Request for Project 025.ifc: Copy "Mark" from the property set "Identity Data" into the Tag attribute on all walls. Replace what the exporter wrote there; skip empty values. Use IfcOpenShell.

First a look at what the model holds.

```python
import ifcopenshell
import ifcopenshell.util.element

model = ifcopenshell.open("Project 025.ifc")
print(model.schema)
walls = model.by_type("IfcWall")
print(len(walls), "walls")
for e in walls[:8]:
    source = ifcopenshell.util.element.get_pset(e, "Identity Data", "Mark")
    target = e.Tag
    print(e.id(), repr(source), repr(target), sep=" | ")
```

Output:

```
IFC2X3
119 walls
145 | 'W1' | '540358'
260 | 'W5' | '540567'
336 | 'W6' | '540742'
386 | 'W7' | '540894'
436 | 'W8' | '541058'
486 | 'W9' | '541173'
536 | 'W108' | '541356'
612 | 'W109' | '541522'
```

```python
import ifcopenshell
import ifcopenshell.util.element

model = ifcopenshell.open("Project 025.ifc")

count = 0
for e in model.by_type("IfcWall"):
    value = ifcopenshell.util.element.get_pset(e, "Identity Data", "Mark")
    current = e.Tag
    if not value or not value.strip() or current == value:
        continue
    e.Tag = value
    count += 1

print(count, "walls updated")

model.write("Project 025-out.ifc")
```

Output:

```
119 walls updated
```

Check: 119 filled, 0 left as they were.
